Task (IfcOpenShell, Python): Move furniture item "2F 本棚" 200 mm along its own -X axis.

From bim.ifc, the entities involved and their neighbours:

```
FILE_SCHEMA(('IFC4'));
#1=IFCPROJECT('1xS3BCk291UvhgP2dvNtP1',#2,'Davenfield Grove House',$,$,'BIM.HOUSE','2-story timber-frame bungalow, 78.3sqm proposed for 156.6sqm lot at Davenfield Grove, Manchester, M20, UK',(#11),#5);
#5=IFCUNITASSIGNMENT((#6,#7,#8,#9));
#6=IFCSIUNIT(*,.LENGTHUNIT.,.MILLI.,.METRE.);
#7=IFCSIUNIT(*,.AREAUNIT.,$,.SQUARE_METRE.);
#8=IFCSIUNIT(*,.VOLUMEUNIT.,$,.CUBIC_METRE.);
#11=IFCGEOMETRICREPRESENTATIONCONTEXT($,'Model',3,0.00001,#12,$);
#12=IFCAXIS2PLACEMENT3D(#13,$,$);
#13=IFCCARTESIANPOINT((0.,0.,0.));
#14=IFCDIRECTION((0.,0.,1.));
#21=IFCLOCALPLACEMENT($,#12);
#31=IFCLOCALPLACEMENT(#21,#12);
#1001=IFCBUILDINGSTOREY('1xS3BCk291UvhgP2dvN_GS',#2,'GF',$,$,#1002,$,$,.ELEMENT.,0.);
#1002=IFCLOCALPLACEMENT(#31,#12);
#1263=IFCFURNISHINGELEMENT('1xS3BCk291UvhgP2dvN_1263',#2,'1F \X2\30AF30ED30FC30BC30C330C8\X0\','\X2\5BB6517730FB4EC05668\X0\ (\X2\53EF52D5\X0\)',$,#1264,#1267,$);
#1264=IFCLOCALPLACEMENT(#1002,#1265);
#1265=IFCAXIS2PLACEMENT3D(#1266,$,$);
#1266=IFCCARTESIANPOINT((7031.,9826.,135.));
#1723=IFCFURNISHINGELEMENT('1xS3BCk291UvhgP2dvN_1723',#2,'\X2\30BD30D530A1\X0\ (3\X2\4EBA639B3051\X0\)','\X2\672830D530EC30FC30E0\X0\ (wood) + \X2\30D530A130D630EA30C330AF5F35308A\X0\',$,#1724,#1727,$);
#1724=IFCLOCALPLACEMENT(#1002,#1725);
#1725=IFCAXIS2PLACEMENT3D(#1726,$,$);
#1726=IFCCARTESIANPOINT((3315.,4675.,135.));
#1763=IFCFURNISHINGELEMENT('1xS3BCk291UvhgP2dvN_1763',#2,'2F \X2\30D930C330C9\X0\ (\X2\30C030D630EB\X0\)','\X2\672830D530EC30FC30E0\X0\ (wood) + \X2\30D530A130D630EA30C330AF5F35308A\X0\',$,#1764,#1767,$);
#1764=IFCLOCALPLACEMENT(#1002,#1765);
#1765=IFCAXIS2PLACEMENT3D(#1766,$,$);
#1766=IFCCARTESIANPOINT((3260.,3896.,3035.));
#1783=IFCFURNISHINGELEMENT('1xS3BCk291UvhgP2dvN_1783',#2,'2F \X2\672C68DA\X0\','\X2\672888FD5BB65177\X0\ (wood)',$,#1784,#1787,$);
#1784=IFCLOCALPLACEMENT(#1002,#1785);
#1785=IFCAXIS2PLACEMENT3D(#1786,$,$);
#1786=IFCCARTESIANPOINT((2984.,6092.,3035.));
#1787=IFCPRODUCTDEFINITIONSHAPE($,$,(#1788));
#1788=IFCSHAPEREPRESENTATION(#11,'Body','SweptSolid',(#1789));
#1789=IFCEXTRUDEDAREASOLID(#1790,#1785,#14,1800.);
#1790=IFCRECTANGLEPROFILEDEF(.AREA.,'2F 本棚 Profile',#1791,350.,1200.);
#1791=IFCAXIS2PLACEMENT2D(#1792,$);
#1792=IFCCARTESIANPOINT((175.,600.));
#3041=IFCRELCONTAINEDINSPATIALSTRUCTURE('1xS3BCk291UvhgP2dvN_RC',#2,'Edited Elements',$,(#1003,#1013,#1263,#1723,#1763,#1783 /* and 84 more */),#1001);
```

```python
import ifcopenshell
import ifcopenshell.api.geometry
import ifcopenshell.util.placement

model = ifcopenshell.open("bim.ifc")

item = model.by_guid("1xS3BCk291UvhgP2dvN_1783")
matrix = ifcopenshell.util.placement.get_local_placement(item.ObjectPlacement)
matrix[:3, 3] -= matrix[:3, 0] * 200.0
ifcopenshell.api.geometry.edit_object_placement(model, product=item, matrix=matrix, is_si=False)

print(ifcopenshell.util.placement.get_local_placement(item.ObjectPlacement).round(3) + 0.0)

model.write("bim_edited.ifc")
```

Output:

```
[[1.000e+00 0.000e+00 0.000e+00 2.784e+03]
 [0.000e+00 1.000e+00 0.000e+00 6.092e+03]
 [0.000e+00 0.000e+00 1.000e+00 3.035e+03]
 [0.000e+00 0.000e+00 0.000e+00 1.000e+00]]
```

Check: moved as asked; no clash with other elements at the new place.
